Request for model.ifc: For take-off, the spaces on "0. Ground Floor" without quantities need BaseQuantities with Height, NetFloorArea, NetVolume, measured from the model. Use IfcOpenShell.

First a look at what the model holds.

```python
import ifcopenshell
import ifcopenshell.util.element
import ifcopenshell.util.unit

model = ifcopenshell.open("model.ifc")
print(model.schema)
for unit_type in ("LENGTHUNIT", "AREAUNIT", "VOLUMEUNIT"):
    print(unit_type, ifcopenshell.util.unit.calculate_unit_scale(model, unit_type))
storey = next(s for s in model.by_type("IfcBuildingStorey") if s.Name == "0. Ground Floor")
spaces = [e for e in ifcopenshell.util.element.get_decomposition(storey) if e.is_a("IfcSpace")]
for e in sorted(spaces, key=lambda e: e.id()):
    print(e.id(), e.is_a(), e.Name, list(ifcopenshell.util.element.get_psets(e, qtos_only=True)), sep=" | ")
```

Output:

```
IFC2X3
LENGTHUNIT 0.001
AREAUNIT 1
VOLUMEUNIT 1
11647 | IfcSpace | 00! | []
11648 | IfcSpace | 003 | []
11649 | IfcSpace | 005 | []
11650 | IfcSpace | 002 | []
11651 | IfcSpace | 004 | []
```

```python
import ifcopenshell
import ifcopenshell.api.pset
import ifcopenshell.geom
import ifcopenshell.util.element
import ifcopenshell.util.shape
import ifcopenshell.util.unit

model = ifcopenshell.open("model.ifc")
unit_scale = ifcopenshell.util.unit.calculate_unit_scale(model)
area_scale = ifcopenshell.util.unit.calculate_unit_scale(model, "AREAUNIT")
volume_scale = ifcopenshell.util.unit.calculate_unit_scale(model, "VOLUMEUNIT")
settings = ifcopenshell.geom.settings()

storey = next(s for s in model.by_type("IfcBuildingStorey") if s.Name == "0. Ground Floor")
spaces = [e for e in ifcopenshell.util.element.get_decomposition(storey) if e.is_a("IfcSpace")]

for e in sorted(spaces, key=lambda e: e.id()):
    if ifcopenshell.util.element.get_psets(e, qtos_only=True, should_inherit=False):
        continue
    # Geometry comes back in metres, in the element's own axes.
    shape = ifcopenshell.geom.create_shape(settings, e)
    values = {
        "Height": ifcopenshell.util.shape.get_z(shape.geometry) / unit_scale,
        "NetFloorArea": ifcopenshell.util.shape.get_footprint_area(shape.geometry) / area_scale,
        "NetVolume": ifcopenshell.util.shape.get_volume(shape.geometry) / volume_scale,
    }
    qto = ifcopenshell.api.pset.add_qto(model, product=e, name="BaseQuantities")
    ifcopenshell.api.pset.edit_qto(model, qto=qto, properties=values)
    print(e.id(), {k: round(v, 3) for k, v in values.items()})

model.write("model-out.ifc")
```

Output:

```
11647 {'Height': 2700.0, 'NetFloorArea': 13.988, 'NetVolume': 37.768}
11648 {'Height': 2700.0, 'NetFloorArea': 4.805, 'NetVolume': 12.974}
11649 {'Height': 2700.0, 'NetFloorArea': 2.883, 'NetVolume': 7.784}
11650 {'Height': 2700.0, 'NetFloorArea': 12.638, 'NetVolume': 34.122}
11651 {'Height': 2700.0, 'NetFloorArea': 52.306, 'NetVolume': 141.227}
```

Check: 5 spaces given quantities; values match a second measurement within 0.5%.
